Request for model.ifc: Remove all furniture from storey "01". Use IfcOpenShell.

First a look at what the model holds.

```python
import ifcopenshell
import ifcopenshell.util.element

model = ifcopenshell.open("model.ifc")
print(model.schema)
storey = next(s for s in model.by_type("IfcBuildingStorey") if s.Name == "01")
furniture = [e for e in ifcopenshell.util.element.get_decomposition(storey) if e.is_a("IfcFurnishingElement")]
seen = {}
for e in furniture:
    element_type = ifcopenshell.util.element.get_type(e)
    name = element_type.Name if element_type not in (None, e) else None
    seen[name] = seen.get(name, 0) + 1
for name, count in sorted(seen.items(), key=str):
    print(count, "x", name)
```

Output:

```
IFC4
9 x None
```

```python
import ifcopenshell
import ifcopenshell.api.root
import ifcopenshell.util.element

model = ifcopenshell.open("model.ifc")

storey = next(s for s in model.by_type("IfcBuildingStorey") if s.Name == "01")
furniture = [e for e in ifcopenshell.util.element.get_decomposition(storey) if e.is_a("IfcFurnishingElement")]

for e in furniture:
    ifcopenshell.api.root.remove_product(model, product=e)
print(len(furniture), "removed")

model.write("model-out.ifc")
```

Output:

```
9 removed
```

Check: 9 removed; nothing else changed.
